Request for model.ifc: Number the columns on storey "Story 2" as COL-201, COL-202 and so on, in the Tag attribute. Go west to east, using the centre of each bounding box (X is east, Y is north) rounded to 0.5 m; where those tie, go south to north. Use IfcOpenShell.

First a look at what the model holds.

```python
import ifcopenshell
import ifcopenshell.util.element
import ifcopenshell.util.placement

model = ifcopenshell.open("model.ifc")
print(model.schema)
storey = next(s for s in model.by_type("IfcBuildingStorey") if s.Name == "Story 2")
columns = [e for e in ifcopenshell.util.element.get_decomposition(storey) if e.is_a("IfcColumn")]
for e in sorted(columns, key=lambda e: e.id()):
    origin = ifcopenshell.util.placement.get_local_placement(e.ObjectPlacement)[:3, 3]
    print(e.id(), e.Tag, e.Name, origin.round(2) + 0.0, sep=" | ")
```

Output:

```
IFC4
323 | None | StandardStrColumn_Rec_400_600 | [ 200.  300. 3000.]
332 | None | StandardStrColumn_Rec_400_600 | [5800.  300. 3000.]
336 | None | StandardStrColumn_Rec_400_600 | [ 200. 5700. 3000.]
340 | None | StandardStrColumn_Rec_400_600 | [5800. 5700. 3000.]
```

```python
import ifcopenshell
import ifcopenshell.geom
import ifcopenshell.util.element
import ifcopenshell.util.shape

model = ifcopenshell.open("model.ifc")
settings = ifcopenshell.geom.settings()
settings.set("use-world-coords", True)


def centre(element):
    shape = ifcopenshell.geom.create_shape(settings, element)
    return ifcopenshell.util.shape.get_bbox_centroid(shape.geometry)


storey = next(s for s in model.by_type("IfcBuildingStorey") if s.Name == "Story 2")
columns = [e for e in ifcopenshell.util.element.get_decomposition(storey) if e.is_a("IfcColumn")]

# Insertion points can sit at a corner or the storey origin, so sort by the geometry (in metres).
centres = {e: centre(e) for e in columns}
columns.sort(key=lambda e: (round(centres[e][0] / 0.5), centres[e][1]))

for i, e in enumerate(columns, start=1):
    number = f"COL-2{i:02d}"
    e.Tag = number
    print(e.id(), number)

model.write("model_v2.ifc")
```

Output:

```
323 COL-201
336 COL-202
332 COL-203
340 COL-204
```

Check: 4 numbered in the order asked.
